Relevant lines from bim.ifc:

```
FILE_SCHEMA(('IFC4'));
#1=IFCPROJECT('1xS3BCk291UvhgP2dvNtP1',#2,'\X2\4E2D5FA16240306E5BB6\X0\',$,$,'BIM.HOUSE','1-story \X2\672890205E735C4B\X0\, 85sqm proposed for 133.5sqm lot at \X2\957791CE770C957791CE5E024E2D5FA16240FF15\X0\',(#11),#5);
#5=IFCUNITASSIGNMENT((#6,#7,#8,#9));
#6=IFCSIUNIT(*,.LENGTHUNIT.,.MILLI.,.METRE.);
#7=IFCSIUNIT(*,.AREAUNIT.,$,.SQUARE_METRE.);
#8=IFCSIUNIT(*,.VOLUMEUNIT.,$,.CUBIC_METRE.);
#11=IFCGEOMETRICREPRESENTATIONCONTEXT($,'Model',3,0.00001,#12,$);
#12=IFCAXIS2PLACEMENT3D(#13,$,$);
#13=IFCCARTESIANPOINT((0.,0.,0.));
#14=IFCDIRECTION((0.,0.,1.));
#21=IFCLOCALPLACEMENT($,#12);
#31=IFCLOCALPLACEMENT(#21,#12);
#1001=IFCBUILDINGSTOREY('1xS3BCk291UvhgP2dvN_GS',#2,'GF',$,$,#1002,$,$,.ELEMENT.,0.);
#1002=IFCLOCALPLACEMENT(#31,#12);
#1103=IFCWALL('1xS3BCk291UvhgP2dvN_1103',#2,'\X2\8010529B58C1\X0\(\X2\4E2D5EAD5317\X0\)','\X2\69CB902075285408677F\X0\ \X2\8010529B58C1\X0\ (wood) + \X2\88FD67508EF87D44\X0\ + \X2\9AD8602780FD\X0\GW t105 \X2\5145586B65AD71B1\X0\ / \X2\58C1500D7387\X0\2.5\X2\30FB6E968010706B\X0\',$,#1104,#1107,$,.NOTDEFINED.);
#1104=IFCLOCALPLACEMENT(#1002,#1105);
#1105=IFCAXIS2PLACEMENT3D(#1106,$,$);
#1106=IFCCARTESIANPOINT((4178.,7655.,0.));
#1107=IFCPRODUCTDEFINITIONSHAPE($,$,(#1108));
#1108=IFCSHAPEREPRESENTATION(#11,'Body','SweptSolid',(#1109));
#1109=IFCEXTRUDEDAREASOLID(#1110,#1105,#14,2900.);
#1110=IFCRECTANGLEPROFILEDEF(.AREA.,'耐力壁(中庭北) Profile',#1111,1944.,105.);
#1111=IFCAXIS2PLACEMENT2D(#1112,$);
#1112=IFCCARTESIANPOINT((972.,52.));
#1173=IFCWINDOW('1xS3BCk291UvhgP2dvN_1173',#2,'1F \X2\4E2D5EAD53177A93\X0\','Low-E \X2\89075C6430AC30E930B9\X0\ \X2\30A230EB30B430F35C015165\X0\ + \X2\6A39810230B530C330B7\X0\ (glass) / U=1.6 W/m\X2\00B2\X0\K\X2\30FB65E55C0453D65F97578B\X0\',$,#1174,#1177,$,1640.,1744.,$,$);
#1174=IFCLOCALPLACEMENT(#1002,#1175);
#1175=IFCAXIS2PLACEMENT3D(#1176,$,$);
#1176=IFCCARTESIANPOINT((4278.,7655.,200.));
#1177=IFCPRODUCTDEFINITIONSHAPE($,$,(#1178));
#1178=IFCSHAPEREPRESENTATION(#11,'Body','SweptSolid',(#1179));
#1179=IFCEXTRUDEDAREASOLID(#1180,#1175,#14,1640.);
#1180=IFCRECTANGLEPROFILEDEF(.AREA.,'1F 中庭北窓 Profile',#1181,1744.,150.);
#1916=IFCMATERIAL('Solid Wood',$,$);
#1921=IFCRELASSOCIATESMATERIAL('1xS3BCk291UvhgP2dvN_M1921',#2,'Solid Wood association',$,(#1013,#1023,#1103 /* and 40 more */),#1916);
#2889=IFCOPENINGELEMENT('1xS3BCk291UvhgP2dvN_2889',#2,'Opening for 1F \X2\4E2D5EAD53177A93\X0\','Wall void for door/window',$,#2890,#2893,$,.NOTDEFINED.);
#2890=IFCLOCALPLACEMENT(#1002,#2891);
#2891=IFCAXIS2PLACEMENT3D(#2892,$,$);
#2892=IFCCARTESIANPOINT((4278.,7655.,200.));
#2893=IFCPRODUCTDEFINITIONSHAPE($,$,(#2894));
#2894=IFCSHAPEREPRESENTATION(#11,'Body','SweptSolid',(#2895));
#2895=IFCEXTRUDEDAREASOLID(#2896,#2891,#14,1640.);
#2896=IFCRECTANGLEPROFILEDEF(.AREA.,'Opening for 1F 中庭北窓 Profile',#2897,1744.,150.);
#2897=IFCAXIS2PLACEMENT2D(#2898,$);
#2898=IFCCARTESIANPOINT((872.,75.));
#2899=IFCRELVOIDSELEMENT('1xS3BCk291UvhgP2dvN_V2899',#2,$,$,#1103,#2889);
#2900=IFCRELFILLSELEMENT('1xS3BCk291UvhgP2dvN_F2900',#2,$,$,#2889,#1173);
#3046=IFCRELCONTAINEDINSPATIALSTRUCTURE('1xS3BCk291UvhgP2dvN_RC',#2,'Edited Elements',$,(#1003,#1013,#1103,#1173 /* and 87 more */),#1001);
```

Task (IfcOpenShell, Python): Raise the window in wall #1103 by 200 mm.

```python
import numpy as np
import ifcopenshell
import ifcopenshell.api.geometry
import ifcopenshell.util.placement
import ifcopenshell.util.unit

model = ifcopenshell.open("bim.ifc")
unit_scale = ifcopenshell.util.unit.calculate_unit_scale(model)

window = model.by_guid("1xS3BCk291UvhgP2dvN_1173")
opening = window.FillsVoids[0].RelatingOpeningElement
dz = 0.2 / unit_scale

shift = np.array([0.0, 0.0, dz])
# The window is not placed relative to its opening, so move both.
for product in (opening, window):
    matrix = ifcopenshell.util.placement.get_local_placement(product.ObjectPlacement)
    matrix[:3, 3] += shift
    ifcopenshell.api.geometry.edit_object_placement(model, product=product, matrix=matrix, is_si=False)

print(f"moved by {dz * unit_scale:+.3f} m")

model.write("bim_rev.ifc")
```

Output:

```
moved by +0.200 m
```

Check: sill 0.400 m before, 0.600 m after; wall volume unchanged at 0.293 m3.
